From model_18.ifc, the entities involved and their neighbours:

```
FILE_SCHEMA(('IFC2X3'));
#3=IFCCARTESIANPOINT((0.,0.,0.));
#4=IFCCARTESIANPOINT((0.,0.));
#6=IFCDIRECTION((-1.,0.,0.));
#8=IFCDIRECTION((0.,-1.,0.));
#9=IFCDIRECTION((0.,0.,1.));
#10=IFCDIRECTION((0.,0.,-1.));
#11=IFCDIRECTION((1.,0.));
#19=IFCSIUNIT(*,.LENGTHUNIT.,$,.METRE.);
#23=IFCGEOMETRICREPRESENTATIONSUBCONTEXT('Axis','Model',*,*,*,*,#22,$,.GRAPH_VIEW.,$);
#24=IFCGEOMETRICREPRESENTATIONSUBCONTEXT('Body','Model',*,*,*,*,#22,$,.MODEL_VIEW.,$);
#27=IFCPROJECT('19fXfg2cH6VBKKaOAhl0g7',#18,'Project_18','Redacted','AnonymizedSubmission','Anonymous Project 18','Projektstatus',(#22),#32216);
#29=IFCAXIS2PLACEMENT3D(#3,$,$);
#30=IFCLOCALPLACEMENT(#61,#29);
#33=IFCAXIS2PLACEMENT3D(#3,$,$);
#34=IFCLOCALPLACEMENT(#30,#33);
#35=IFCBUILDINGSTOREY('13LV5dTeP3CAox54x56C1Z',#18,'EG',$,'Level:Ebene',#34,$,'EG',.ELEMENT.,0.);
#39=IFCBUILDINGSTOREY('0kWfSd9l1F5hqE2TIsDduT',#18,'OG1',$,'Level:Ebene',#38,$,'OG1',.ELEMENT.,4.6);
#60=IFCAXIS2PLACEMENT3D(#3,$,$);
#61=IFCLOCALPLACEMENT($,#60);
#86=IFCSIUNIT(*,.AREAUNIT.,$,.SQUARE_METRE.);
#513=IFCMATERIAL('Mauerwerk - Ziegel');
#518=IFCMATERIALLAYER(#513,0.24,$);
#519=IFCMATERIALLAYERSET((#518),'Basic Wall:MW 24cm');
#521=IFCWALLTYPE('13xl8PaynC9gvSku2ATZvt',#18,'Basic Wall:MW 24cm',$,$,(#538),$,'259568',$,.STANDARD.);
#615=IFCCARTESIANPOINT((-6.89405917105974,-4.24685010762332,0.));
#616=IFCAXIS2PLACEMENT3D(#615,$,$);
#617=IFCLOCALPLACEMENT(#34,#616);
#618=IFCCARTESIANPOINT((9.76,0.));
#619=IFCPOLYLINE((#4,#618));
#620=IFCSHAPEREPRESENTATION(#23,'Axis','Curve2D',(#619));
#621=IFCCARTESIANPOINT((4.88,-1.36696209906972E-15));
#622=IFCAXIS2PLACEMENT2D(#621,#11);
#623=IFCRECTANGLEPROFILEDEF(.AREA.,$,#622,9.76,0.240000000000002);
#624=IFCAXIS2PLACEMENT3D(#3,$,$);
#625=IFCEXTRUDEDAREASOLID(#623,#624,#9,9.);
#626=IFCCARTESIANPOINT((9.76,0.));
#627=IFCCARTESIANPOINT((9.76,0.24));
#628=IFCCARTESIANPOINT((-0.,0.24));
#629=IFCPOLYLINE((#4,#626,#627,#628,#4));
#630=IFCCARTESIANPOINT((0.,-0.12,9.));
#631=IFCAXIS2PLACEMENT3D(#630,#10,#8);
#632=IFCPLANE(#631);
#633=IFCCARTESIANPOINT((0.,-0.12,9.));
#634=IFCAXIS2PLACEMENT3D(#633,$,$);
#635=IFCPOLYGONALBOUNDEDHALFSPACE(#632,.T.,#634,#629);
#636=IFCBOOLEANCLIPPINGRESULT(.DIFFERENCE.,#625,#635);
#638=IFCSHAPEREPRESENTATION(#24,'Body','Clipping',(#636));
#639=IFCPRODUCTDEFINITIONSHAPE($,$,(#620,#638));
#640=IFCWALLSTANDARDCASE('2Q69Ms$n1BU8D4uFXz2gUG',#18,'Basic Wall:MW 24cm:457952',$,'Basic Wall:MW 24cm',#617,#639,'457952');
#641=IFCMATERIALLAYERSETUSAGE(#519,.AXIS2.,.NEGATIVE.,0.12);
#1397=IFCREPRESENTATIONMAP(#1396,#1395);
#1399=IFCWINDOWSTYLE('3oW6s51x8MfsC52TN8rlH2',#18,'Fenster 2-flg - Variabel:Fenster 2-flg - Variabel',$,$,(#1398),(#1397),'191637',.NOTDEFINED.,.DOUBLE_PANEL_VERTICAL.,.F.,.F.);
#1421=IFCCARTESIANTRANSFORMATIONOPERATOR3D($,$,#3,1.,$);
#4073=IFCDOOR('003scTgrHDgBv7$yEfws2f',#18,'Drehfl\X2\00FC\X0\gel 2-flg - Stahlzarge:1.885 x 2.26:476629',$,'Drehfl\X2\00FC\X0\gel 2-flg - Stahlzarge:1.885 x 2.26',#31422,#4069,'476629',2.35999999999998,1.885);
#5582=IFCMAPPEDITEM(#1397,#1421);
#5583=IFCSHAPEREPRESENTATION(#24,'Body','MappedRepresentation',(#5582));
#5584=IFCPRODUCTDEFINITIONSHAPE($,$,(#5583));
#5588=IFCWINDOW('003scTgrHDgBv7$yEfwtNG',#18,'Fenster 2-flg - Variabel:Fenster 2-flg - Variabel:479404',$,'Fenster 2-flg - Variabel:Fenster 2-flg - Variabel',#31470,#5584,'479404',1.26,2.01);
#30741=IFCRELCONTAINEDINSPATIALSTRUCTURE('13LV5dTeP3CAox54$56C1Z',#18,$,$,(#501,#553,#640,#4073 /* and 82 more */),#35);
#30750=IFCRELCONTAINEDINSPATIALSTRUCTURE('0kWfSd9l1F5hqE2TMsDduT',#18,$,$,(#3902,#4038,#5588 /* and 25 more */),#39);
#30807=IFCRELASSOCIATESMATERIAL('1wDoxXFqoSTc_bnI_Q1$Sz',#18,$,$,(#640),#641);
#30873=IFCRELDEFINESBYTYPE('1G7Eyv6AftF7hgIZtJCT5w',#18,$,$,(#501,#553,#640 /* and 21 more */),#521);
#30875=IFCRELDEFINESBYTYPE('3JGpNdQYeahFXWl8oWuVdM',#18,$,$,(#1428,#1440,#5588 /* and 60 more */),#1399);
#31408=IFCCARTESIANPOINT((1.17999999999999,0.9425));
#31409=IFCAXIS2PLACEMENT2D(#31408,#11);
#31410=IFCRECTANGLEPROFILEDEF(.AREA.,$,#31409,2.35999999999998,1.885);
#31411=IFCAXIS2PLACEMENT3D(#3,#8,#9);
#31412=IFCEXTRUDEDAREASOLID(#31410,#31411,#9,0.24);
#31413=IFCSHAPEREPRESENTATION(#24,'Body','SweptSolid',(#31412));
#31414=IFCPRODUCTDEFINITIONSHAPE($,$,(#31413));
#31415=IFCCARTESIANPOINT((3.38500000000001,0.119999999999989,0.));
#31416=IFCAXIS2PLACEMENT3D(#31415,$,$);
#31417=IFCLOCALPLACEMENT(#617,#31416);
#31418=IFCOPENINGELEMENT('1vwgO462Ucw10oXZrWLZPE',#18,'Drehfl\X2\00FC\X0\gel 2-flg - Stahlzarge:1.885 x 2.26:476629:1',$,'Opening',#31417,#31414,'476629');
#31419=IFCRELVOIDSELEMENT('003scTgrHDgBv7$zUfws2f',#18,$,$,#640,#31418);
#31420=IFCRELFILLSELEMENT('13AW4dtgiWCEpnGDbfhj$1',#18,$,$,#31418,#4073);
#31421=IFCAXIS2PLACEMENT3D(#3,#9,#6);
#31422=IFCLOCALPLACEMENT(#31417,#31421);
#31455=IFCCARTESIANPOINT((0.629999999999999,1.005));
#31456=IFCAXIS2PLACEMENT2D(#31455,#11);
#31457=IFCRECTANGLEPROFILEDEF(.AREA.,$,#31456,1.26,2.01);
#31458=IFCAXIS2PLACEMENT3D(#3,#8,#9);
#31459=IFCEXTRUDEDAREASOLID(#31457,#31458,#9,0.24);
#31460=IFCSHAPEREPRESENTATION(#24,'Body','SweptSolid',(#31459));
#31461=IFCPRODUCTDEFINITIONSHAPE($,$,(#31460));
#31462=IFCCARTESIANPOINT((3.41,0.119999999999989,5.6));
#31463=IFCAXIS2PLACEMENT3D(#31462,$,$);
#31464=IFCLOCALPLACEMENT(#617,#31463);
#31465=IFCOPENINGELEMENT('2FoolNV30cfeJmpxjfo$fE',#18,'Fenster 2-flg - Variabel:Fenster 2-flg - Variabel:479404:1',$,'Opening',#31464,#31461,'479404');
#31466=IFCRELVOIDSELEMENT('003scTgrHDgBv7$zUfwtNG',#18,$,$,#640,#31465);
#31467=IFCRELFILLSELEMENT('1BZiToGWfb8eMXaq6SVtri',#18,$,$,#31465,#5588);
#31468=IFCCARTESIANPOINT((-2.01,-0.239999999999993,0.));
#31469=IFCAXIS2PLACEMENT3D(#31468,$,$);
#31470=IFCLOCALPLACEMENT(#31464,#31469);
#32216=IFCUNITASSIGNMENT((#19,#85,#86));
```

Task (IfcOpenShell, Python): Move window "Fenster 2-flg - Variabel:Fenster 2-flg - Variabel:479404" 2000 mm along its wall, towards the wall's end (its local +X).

```python
import ifcopenshell
import ifcopenshell.api.geometry
import ifcopenshell.util.placement

model = ifcopenshell.open("model_18.ifc")

window = model.by_guid("003scTgrHDgBv7$yEfwtNG")
opening = window.FillsVoids[0].RelatingOpeningElement
wall = opening.VoidsElements[0].RelatingBuildingElement

wall_matrix = ifcopenshell.util.placement.get_local_placement(wall.ObjectPlacement)
shift = wall_matrix[:3, 0] * 2.0
before = ifcopenshell.util.placement.get_local_placement(window.ObjectPlacement)[:3, 3].copy()

# The window is placed relative to its opening, so it follows when the opening moves.
matrix = ifcopenshell.util.placement.get_local_placement(opening.ObjectPlacement)
matrix[:3, 3] += shift
ifcopenshell.api.geometry.edit_object_placement(
    model, product=opening, matrix=matrix, is_si=False, should_transform_children=True
)

after = ifcopenshell.util.placement.get_local_placement(window.ObjectPlacement)[:3, 3]
print("window moved by", (after - before).round(3) + 0.0)

model.write("model_18_updated.ifc")
```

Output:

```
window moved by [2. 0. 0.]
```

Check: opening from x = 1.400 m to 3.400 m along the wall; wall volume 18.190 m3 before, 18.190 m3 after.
